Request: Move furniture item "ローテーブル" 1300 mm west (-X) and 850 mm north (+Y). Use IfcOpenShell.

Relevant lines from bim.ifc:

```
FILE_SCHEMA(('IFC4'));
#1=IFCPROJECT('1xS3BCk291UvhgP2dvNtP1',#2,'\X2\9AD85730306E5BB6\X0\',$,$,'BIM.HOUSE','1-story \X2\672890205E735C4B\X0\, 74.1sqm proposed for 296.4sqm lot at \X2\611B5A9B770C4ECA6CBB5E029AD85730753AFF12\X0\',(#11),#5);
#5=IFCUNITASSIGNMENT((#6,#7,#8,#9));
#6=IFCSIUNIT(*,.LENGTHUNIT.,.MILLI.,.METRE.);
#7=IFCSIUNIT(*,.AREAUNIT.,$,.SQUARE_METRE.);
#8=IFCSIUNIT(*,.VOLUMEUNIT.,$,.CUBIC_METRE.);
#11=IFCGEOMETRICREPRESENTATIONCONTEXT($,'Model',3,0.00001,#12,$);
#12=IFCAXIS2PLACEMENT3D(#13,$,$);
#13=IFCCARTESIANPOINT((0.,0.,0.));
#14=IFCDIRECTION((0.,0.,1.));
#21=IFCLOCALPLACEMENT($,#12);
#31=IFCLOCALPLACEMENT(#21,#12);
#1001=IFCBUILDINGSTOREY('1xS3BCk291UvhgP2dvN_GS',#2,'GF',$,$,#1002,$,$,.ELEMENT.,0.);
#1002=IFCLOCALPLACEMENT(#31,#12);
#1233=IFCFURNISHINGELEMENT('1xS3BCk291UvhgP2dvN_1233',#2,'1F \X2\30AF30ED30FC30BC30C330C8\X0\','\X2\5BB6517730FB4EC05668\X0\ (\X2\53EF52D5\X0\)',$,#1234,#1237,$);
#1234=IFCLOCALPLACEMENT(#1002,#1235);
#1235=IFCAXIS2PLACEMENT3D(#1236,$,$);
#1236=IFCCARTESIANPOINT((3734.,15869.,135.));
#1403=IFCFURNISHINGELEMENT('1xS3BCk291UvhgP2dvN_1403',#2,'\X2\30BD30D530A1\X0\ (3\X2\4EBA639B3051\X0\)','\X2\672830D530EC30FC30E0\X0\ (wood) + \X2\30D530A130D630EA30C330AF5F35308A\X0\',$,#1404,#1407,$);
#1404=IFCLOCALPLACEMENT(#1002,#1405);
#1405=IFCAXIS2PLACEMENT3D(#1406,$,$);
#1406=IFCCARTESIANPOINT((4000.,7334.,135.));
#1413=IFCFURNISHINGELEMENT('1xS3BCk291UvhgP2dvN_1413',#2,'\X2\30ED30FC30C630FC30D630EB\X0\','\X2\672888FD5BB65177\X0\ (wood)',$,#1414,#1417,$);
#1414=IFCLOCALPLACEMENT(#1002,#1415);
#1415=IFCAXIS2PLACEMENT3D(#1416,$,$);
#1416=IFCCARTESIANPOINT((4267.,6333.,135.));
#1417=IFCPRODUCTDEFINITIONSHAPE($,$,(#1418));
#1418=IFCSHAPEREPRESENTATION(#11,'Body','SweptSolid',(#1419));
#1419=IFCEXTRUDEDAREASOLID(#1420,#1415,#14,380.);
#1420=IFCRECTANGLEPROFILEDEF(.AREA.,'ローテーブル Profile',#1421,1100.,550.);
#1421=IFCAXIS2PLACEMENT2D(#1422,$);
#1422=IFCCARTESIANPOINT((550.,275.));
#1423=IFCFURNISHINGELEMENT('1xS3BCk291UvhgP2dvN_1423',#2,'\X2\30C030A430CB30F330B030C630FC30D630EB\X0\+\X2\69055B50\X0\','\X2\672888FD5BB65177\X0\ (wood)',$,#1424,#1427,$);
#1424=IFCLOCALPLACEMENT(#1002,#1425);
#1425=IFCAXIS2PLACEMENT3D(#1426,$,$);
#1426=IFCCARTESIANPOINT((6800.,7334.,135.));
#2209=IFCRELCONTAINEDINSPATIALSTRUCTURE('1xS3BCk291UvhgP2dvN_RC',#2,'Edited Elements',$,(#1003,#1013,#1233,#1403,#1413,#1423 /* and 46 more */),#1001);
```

```python
import ifcopenshell
import ifcopenshell.api.geometry
import ifcopenshell.util.placement
import ifcopenshell.util.unit

model = ifcopenshell.open("bim.ifc")
unit_scale = ifcopenshell.util.unit.calculate_unit_scale(model)

item = model.by_guid("1xS3BCk291UvhgP2dvN_1413")
matrix = ifcopenshell.util.placement.get_local_placement(item.ObjectPlacement)
matrix[0, 3] -= 1.3 / unit_scale
matrix[1, 3] += 0.85 / unit_scale
ifcopenshell.api.geometry.edit_object_placement(model, product=item, matrix=matrix, is_si=False)

print(ifcopenshell.util.placement.get_local_placement(item.ObjectPlacement).round(3) + 0.0)

model.write("bim_v2.ifc")
```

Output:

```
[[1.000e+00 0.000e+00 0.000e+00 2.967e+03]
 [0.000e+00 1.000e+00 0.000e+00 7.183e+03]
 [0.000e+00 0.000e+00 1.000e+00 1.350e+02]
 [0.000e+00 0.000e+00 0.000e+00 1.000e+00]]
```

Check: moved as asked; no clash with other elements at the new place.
